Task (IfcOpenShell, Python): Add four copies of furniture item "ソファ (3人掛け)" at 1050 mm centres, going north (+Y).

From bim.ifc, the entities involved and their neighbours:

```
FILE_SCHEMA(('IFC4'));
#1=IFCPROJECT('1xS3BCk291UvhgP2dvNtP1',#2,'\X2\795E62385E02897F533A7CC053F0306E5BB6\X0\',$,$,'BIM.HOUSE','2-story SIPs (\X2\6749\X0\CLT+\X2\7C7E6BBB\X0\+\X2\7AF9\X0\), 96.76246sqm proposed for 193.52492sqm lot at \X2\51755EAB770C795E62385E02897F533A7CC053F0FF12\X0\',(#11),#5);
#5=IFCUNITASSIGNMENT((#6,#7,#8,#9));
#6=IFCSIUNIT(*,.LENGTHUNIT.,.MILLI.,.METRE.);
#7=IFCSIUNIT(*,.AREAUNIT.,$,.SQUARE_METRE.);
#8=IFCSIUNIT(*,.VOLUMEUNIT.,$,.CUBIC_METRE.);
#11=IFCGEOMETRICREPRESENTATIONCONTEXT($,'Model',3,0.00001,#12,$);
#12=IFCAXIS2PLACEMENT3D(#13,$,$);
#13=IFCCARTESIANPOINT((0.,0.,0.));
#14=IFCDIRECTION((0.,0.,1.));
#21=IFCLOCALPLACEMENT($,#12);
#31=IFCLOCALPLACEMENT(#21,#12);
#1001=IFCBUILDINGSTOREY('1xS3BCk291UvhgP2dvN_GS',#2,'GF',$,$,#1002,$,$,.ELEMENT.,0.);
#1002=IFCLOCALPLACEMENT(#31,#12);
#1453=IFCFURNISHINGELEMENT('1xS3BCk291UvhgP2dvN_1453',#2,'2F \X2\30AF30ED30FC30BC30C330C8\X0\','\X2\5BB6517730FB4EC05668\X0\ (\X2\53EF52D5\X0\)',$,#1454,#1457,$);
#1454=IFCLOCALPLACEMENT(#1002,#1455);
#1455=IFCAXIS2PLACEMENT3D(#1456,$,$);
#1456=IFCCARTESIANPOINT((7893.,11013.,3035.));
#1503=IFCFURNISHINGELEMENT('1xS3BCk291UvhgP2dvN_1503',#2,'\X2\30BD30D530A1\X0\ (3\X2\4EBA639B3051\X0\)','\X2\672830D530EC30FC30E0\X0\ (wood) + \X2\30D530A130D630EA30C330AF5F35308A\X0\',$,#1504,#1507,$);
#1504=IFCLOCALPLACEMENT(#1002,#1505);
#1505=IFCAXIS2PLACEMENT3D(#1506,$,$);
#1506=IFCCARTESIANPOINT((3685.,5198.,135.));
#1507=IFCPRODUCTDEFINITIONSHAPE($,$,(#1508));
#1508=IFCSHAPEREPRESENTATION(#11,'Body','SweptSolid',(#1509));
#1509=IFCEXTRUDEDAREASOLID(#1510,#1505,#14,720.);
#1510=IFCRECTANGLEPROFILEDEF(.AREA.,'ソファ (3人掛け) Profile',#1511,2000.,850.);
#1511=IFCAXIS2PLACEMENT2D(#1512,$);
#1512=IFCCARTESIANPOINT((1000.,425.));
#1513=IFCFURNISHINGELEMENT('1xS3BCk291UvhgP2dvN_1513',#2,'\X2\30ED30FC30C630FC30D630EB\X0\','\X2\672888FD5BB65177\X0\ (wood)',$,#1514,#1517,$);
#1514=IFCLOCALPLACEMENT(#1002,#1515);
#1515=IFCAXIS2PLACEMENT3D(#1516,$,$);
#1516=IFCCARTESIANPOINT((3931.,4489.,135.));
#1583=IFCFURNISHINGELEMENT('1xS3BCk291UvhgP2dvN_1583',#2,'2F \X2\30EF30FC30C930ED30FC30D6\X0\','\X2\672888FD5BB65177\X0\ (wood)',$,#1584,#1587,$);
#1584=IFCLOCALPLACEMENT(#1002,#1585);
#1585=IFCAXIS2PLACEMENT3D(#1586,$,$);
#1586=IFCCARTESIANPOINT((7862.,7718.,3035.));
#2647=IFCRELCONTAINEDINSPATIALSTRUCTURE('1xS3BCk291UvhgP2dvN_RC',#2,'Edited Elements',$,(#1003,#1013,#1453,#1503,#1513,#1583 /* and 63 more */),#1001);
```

```python
import numpy as np
import ifcopenshell
import ifcopenshell.api.geometry
import ifcopenshell.api.root
import ifcopenshell.util.element
import ifcopenshell.util.placement

model = ifcopenshell.open("bim.ifc")


def reuse_history(source, copy):
    """copy_class also copies each property set's owner history, people and application; keep the originals."""
    for rel in copy.IsDefinedBy:
        if rel.is_a("IfcRelDefinesByProperties") and (history := rel.RelatingPropertyDefinition.OwnerHistory):
            rel.RelatingPropertyDefinition.OwnerHistory = source.OwnerHistory
            ifcopenshell.util.element.remove_deep2(model, history)


source = model.by_guid("1xS3BCk291UvhgP2dvN_1503")
base = ifcopenshell.util.placement.get_local_placement(source.ObjectPlacement)
step = np.array([0.0, 1.0, 0.0]) * 1050.0

for i in range(1, 5):
    copy = ifcopenshell.api.root.copy_class(model, product=source)
    copy.Representation = ifcopenshell.util.element.copy_deep(
        model, source.Representation, exclude=["IfcGeometricRepresentationContext", "IfcRepresentationMap"]
    )
    reuse_history(source, copy)
    matrix = base.copy()
    matrix[:3, 3] += i * step
    print("added at", matrix[:3, 3].round(3) + 0.0)
    ifcopenshell.api.geometry.edit_object_placement(model, product=copy, matrix=matrix, is_si=False)

model.write("bim_updated.ifc")
```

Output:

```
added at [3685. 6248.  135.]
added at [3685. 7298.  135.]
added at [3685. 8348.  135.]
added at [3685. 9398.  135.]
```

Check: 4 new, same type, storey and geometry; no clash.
